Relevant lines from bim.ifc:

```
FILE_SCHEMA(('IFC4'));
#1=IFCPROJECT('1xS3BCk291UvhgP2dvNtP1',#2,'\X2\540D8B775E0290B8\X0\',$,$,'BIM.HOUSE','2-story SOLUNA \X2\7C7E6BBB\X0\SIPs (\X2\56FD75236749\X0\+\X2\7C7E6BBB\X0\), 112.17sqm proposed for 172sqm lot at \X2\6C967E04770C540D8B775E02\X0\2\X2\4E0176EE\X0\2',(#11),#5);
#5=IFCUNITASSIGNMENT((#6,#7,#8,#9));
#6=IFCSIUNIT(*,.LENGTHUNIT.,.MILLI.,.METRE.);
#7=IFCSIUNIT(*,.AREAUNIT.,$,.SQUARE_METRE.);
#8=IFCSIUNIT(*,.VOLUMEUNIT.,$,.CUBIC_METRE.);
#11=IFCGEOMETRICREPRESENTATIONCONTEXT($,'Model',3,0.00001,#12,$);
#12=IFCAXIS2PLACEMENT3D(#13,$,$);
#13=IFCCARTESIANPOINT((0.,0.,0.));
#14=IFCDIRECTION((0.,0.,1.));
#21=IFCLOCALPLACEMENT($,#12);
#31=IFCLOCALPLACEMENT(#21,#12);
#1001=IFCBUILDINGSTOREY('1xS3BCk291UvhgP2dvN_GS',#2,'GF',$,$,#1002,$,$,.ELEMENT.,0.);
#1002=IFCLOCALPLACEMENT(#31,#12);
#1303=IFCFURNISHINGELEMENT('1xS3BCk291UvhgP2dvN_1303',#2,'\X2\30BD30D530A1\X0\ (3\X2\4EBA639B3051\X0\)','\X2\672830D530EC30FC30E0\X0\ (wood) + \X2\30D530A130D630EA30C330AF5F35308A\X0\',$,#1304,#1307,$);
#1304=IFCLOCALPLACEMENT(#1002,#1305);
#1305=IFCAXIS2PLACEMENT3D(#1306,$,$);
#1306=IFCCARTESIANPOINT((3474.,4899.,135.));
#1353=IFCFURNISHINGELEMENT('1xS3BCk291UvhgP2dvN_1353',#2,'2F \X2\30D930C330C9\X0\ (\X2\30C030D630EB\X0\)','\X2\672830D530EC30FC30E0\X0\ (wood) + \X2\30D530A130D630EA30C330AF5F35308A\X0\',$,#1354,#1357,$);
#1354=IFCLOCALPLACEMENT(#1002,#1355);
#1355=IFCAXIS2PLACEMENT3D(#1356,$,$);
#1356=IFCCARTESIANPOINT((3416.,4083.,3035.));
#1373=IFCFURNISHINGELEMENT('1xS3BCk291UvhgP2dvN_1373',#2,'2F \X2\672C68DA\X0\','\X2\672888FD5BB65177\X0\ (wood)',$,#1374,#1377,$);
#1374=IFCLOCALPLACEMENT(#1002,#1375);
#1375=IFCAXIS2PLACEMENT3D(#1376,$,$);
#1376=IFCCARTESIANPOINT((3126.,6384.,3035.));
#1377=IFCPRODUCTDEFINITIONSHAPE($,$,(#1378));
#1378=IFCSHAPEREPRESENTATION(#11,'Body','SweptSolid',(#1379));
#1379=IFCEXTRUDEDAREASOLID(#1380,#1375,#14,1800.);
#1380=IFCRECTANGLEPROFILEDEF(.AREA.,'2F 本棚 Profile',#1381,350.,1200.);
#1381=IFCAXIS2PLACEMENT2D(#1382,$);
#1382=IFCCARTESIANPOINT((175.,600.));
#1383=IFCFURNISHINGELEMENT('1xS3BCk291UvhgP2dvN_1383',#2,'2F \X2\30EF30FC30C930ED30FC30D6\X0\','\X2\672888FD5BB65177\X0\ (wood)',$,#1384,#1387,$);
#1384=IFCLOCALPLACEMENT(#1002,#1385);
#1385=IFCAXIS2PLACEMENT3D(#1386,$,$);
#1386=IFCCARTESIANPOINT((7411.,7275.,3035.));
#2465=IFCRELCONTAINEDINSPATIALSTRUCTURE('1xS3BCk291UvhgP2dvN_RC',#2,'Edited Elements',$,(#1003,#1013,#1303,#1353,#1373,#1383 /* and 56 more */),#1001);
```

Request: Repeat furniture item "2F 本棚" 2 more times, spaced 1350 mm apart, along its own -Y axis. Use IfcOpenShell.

```python
import ifcopenshell
import ifcopenshell.api.geometry
import ifcopenshell.api.root
import ifcopenshell.util.element
import ifcopenshell.util.placement
import ifcopenshell.util.unit

model = ifcopenshell.open("bim.ifc")
unit_scale = ifcopenshell.util.unit.calculate_unit_scale(model)


def reuse_history(source, copy):
    """copy_class also copies each property set's owner history, people and application; keep the originals."""
    for rel in copy.IsDefinedBy:
        if rel.is_a("IfcRelDefinesByProperties") and (history := rel.RelatingPropertyDefinition.OwnerHistory):
            rel.RelatingPropertyDefinition.OwnerHistory = source.OwnerHistory
            ifcopenshell.util.element.remove_deep2(model, history)


source = model.by_guid("1xS3BCk291UvhgP2dvN_1373")
base = ifcopenshell.util.placement.get_local_placement(source.ObjectPlacement)
step = -base[:3, 1] * 1.35 / unit_scale

for i in range(1, 3):
    copy = ifcopenshell.api.root.copy_class(model, product=source)
    copy.Representation = ifcopenshell.util.element.copy_deep(
        model, source.Representation, exclude=["IfcGeometricRepresentationContext", "IfcRepresentationMap"]
    )
    reuse_history(source, copy)
    matrix = base.copy()
    matrix[:3, 3] += i * step
    print("added at", matrix[:3, 3].round(3) + 0.0)
    ifcopenshell.api.geometry.edit_object_placement(model, product=copy, matrix=matrix, is_si=False)

model.write("bim_edited.ifc")
```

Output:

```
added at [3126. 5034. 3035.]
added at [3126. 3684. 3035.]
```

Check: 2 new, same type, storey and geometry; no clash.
